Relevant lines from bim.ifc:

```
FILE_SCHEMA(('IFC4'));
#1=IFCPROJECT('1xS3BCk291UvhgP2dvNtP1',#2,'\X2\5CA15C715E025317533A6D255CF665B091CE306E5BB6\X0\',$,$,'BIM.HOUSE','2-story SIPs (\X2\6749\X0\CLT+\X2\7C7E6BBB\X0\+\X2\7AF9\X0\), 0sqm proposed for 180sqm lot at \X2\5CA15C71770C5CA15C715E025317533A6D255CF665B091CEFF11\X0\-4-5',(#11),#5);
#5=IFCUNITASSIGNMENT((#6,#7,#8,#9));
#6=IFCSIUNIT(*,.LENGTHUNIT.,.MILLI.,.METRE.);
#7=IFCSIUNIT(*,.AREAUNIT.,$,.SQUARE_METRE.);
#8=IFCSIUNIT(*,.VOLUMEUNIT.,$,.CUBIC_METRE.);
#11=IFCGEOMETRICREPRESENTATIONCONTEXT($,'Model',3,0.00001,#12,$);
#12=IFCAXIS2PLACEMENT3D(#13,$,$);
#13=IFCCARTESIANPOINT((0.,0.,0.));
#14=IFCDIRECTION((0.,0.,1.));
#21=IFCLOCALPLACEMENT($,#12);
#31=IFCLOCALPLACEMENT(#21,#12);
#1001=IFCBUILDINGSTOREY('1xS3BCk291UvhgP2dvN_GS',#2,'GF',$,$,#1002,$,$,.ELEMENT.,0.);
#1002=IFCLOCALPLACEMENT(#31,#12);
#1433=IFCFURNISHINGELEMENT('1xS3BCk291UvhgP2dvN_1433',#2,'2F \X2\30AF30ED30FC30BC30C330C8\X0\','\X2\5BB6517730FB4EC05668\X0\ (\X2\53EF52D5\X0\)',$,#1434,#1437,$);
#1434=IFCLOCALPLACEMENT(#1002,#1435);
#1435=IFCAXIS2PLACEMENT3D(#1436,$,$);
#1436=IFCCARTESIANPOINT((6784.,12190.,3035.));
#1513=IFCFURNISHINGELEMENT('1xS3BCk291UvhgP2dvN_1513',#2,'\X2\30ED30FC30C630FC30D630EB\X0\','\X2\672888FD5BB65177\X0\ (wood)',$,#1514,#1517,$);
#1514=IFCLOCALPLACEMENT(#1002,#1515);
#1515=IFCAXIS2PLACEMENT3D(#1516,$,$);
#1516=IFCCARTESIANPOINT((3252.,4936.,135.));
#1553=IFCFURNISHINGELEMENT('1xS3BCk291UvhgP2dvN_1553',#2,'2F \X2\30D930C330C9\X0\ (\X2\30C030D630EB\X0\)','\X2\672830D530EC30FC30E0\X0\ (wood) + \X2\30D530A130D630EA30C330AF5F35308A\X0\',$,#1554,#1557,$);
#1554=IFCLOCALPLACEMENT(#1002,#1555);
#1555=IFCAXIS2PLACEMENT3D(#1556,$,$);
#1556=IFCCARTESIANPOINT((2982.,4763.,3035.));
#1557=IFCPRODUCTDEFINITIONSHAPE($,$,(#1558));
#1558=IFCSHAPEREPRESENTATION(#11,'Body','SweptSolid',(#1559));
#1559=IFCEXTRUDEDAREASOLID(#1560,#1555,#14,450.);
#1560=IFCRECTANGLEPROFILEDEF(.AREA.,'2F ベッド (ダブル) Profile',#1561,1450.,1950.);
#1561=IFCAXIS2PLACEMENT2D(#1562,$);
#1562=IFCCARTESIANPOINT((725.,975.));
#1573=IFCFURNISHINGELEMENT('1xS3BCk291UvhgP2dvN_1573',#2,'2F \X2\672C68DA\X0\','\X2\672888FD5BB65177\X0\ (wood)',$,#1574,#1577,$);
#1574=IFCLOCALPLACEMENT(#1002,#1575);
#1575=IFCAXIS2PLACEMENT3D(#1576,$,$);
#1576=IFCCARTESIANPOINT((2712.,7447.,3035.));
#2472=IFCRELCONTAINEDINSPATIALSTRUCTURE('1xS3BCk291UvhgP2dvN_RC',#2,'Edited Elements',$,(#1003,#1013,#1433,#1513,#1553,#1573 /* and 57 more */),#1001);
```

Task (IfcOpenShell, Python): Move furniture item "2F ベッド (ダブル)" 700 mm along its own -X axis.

```python
import ifcopenshell
import ifcopenshell.api.geometry
import ifcopenshell.util.placement
import ifcopenshell.util.unit

model = ifcopenshell.open("bim.ifc")
unit_scale = ifcopenshell.util.unit.calculate_unit_scale(model)

item = model.by_guid("1xS3BCk291UvhgP2dvN_1553")
matrix = ifcopenshell.util.placement.get_local_placement(item.ObjectPlacement)
matrix[:3, 3] -= matrix[:3, 0] * 0.7 / unit_scale
ifcopenshell.api.geometry.edit_object_placement(model, product=item, matrix=matrix, is_si=False)

print(ifcopenshell.util.placement.get_local_placement(item.ObjectPlacement).round(3) + 0.0)

model.write("bim_v2.ifc")
```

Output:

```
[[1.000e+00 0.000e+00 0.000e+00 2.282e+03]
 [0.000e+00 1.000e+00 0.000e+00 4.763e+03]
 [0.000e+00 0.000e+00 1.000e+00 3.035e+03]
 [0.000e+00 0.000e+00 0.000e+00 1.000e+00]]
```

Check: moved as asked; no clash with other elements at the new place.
